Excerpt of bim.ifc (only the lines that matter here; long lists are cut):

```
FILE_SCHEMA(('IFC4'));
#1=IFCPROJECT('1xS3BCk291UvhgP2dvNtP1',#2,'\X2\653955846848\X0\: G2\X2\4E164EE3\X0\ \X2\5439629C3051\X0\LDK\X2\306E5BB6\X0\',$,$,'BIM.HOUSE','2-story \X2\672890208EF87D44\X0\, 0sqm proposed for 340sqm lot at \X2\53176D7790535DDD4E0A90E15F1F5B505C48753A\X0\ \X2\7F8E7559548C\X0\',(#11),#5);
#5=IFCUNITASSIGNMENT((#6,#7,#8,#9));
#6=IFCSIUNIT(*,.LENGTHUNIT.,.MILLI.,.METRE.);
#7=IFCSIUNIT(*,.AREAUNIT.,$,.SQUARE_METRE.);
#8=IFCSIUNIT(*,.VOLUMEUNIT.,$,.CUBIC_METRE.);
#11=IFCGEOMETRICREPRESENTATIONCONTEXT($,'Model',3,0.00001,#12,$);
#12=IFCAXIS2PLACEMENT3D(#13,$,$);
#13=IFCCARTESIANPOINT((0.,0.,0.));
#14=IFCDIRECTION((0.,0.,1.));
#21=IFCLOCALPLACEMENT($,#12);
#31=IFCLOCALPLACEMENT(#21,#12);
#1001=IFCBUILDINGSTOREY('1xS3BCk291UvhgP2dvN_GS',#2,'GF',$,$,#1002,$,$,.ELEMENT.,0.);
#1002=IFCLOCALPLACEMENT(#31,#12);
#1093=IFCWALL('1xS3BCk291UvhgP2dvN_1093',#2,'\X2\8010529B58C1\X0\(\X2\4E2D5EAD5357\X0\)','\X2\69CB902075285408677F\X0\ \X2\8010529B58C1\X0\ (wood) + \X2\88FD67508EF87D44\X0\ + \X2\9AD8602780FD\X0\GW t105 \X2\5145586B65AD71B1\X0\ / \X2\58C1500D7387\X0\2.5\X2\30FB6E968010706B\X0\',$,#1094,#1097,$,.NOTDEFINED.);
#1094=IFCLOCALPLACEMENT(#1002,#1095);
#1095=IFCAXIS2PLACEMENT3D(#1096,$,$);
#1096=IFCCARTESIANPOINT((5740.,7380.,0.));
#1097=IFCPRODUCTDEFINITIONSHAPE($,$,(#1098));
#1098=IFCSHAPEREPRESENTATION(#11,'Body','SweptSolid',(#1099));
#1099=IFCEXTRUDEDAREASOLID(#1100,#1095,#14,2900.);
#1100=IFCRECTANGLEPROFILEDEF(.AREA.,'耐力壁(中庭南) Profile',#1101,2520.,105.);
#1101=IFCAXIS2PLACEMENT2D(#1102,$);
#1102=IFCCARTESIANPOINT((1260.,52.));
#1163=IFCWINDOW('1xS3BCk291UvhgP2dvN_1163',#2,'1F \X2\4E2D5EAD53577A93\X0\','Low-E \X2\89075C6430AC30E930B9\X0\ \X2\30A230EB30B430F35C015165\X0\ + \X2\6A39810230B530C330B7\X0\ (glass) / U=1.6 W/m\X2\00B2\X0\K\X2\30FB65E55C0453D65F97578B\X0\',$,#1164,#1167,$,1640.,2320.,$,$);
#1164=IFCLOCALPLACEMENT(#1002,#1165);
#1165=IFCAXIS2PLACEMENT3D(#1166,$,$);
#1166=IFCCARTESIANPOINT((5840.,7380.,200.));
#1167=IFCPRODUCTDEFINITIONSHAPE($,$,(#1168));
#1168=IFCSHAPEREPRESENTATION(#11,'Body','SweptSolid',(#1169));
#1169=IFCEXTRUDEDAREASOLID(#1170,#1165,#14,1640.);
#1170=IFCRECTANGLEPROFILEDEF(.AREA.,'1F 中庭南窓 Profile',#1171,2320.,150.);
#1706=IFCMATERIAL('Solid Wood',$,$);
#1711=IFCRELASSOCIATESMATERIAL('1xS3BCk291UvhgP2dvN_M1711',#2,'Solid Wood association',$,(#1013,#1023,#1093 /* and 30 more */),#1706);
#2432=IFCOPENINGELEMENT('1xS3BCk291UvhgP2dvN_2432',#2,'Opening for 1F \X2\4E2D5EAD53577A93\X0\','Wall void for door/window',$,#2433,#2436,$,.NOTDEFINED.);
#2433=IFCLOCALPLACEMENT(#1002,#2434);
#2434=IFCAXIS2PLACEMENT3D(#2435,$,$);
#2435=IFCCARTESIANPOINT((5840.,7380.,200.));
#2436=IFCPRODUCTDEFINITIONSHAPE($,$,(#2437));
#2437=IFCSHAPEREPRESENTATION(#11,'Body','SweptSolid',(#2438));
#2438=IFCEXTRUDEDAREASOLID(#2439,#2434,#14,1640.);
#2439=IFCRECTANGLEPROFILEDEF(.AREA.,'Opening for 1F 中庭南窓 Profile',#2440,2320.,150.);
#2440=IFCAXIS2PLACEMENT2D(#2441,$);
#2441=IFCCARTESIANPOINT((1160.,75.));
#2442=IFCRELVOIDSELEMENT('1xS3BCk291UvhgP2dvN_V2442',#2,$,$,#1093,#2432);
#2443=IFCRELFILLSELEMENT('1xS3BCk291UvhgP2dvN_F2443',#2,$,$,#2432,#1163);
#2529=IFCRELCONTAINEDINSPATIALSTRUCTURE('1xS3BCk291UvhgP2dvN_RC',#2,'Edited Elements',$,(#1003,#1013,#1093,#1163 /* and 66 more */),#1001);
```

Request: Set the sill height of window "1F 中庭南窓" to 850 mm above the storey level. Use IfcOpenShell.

```python
import numpy as np
import ifcopenshell
import ifcopenshell.api.geometry
import ifcopenshell.geom
import ifcopenshell.util.element
import ifcopenshell.util.placement
import ifcopenshell.util.shape
import ifcopenshell.util.unit

model = ifcopenshell.open("bim.ifc")
unit_scale = ifcopenshell.util.unit.calculate_unit_scale(model)

window = model.by_id(1163)
opening = window.FillsVoids[0].RelatingOpeningElement
storey = ifcopenshell.util.element.get_container(window, ifc_class="IfcBuildingStorey")
level = ifcopenshell.util.placement.get_local_placement(storey.ObjectPlacement)[2, 3]

# The opening's origin need not be at the sill, so measure its lowest point.
shape = ifcopenshell.geom.create_shape(ifcopenshell.geom.settings(), opening)
bottom = ifcopenshell.util.shape.get_shape_bottom_elevation(shape, shape.geometry) / unit_scale
dz = level + 0.85 / unit_scale - bottom

shift = np.array([0.0, 0.0, dz])
# The window is not placed relative to its opening, so move both.
for product in (opening, window):
    matrix = ifcopenshell.util.placement.get_local_placement(product.ObjectPlacement)
    matrix[:3, 3] += shift
    ifcopenshell.api.geometry.edit_object_placement(model, product=product, matrix=matrix, is_si=False)

print(f"moved by {dz * unit_scale:+.3f} m")

model.write("bim_v2.ifc")
```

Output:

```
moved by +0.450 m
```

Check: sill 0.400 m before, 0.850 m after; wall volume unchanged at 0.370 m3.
